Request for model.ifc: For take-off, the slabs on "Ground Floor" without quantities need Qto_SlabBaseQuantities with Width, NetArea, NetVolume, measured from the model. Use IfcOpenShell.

First a look at what the model holds.

```python
import ifcopenshell
import ifcopenshell.util.element
import ifcopenshell.util.unit

model = ifcopenshell.open("model.ifc")
print(model.schema)
for unit_type in ("LENGTHUNIT", "AREAUNIT", "VOLUMEUNIT"):
    print(unit_type, ifcopenshell.util.unit.calculate_unit_scale(model, unit_type))
storey = next(s for s in model.by_type("IfcBuildingStorey") if s.Name == "Ground Floor")
slabs = [e for e in ifcopenshell.util.element.get_decomposition(storey) if e.is_a("IfcSlab")]
for e in sorted(slabs, key=lambda e: e.id()):
    print(e.id(), e.is_a(), e.Name, list(ifcopenshell.util.element.get_psets(e, qtos_only=True)), sep=" | ")
```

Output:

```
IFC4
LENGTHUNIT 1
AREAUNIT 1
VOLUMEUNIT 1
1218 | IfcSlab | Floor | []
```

```python
import ifcopenshell
import ifcopenshell.api.pset
import ifcopenshell.geom
import ifcopenshell.util.element
import ifcopenshell.util.shape
import ifcopenshell.util.unit

model = ifcopenshell.open("model.ifc")
unit_scale = ifcopenshell.util.unit.calculate_unit_scale(model)
area_scale = ifcopenshell.util.unit.calculate_unit_scale(model, "AREAUNIT")
volume_scale = ifcopenshell.util.unit.calculate_unit_scale(model, "VOLUMEUNIT")
settings = ifcopenshell.geom.settings()

storey = next(s for s in model.by_type("IfcBuildingStorey") if s.Name == "Ground Floor")
slabs = [e for e in ifcopenshell.util.element.get_decomposition(storey) if e.is_a("IfcSlab")]

for e in sorted(slabs, key=lambda e: e.id()):
    if ifcopenshell.util.element.get_psets(e, qtos_only=True, should_inherit=False):
        continue
    # Geometry comes back in metres, in the element's own axes.
    shape = ifcopenshell.geom.create_shape(settings, e)
    values = {
        "Width": ifcopenshell.util.shape.get_z(shape.geometry) / unit_scale,
        "NetArea": ifcopenshell.util.shape.get_footprint_area(shape.geometry) / area_scale,
        "NetVolume": ifcopenshell.util.shape.get_volume(shape.geometry) / volume_scale,
    }
    qto = ifcopenshell.api.pset.add_qto(model, product=e, name="Qto_SlabBaseQuantities")
    ifcopenshell.api.pset.edit_qto(model, qto=qto, properties=values)
    print(e.id(), {k: round(v, 3) for k, v in values.items()})

model.write("model_v2.ifc")
```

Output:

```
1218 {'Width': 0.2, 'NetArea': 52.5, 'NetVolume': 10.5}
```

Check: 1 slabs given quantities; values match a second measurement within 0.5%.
